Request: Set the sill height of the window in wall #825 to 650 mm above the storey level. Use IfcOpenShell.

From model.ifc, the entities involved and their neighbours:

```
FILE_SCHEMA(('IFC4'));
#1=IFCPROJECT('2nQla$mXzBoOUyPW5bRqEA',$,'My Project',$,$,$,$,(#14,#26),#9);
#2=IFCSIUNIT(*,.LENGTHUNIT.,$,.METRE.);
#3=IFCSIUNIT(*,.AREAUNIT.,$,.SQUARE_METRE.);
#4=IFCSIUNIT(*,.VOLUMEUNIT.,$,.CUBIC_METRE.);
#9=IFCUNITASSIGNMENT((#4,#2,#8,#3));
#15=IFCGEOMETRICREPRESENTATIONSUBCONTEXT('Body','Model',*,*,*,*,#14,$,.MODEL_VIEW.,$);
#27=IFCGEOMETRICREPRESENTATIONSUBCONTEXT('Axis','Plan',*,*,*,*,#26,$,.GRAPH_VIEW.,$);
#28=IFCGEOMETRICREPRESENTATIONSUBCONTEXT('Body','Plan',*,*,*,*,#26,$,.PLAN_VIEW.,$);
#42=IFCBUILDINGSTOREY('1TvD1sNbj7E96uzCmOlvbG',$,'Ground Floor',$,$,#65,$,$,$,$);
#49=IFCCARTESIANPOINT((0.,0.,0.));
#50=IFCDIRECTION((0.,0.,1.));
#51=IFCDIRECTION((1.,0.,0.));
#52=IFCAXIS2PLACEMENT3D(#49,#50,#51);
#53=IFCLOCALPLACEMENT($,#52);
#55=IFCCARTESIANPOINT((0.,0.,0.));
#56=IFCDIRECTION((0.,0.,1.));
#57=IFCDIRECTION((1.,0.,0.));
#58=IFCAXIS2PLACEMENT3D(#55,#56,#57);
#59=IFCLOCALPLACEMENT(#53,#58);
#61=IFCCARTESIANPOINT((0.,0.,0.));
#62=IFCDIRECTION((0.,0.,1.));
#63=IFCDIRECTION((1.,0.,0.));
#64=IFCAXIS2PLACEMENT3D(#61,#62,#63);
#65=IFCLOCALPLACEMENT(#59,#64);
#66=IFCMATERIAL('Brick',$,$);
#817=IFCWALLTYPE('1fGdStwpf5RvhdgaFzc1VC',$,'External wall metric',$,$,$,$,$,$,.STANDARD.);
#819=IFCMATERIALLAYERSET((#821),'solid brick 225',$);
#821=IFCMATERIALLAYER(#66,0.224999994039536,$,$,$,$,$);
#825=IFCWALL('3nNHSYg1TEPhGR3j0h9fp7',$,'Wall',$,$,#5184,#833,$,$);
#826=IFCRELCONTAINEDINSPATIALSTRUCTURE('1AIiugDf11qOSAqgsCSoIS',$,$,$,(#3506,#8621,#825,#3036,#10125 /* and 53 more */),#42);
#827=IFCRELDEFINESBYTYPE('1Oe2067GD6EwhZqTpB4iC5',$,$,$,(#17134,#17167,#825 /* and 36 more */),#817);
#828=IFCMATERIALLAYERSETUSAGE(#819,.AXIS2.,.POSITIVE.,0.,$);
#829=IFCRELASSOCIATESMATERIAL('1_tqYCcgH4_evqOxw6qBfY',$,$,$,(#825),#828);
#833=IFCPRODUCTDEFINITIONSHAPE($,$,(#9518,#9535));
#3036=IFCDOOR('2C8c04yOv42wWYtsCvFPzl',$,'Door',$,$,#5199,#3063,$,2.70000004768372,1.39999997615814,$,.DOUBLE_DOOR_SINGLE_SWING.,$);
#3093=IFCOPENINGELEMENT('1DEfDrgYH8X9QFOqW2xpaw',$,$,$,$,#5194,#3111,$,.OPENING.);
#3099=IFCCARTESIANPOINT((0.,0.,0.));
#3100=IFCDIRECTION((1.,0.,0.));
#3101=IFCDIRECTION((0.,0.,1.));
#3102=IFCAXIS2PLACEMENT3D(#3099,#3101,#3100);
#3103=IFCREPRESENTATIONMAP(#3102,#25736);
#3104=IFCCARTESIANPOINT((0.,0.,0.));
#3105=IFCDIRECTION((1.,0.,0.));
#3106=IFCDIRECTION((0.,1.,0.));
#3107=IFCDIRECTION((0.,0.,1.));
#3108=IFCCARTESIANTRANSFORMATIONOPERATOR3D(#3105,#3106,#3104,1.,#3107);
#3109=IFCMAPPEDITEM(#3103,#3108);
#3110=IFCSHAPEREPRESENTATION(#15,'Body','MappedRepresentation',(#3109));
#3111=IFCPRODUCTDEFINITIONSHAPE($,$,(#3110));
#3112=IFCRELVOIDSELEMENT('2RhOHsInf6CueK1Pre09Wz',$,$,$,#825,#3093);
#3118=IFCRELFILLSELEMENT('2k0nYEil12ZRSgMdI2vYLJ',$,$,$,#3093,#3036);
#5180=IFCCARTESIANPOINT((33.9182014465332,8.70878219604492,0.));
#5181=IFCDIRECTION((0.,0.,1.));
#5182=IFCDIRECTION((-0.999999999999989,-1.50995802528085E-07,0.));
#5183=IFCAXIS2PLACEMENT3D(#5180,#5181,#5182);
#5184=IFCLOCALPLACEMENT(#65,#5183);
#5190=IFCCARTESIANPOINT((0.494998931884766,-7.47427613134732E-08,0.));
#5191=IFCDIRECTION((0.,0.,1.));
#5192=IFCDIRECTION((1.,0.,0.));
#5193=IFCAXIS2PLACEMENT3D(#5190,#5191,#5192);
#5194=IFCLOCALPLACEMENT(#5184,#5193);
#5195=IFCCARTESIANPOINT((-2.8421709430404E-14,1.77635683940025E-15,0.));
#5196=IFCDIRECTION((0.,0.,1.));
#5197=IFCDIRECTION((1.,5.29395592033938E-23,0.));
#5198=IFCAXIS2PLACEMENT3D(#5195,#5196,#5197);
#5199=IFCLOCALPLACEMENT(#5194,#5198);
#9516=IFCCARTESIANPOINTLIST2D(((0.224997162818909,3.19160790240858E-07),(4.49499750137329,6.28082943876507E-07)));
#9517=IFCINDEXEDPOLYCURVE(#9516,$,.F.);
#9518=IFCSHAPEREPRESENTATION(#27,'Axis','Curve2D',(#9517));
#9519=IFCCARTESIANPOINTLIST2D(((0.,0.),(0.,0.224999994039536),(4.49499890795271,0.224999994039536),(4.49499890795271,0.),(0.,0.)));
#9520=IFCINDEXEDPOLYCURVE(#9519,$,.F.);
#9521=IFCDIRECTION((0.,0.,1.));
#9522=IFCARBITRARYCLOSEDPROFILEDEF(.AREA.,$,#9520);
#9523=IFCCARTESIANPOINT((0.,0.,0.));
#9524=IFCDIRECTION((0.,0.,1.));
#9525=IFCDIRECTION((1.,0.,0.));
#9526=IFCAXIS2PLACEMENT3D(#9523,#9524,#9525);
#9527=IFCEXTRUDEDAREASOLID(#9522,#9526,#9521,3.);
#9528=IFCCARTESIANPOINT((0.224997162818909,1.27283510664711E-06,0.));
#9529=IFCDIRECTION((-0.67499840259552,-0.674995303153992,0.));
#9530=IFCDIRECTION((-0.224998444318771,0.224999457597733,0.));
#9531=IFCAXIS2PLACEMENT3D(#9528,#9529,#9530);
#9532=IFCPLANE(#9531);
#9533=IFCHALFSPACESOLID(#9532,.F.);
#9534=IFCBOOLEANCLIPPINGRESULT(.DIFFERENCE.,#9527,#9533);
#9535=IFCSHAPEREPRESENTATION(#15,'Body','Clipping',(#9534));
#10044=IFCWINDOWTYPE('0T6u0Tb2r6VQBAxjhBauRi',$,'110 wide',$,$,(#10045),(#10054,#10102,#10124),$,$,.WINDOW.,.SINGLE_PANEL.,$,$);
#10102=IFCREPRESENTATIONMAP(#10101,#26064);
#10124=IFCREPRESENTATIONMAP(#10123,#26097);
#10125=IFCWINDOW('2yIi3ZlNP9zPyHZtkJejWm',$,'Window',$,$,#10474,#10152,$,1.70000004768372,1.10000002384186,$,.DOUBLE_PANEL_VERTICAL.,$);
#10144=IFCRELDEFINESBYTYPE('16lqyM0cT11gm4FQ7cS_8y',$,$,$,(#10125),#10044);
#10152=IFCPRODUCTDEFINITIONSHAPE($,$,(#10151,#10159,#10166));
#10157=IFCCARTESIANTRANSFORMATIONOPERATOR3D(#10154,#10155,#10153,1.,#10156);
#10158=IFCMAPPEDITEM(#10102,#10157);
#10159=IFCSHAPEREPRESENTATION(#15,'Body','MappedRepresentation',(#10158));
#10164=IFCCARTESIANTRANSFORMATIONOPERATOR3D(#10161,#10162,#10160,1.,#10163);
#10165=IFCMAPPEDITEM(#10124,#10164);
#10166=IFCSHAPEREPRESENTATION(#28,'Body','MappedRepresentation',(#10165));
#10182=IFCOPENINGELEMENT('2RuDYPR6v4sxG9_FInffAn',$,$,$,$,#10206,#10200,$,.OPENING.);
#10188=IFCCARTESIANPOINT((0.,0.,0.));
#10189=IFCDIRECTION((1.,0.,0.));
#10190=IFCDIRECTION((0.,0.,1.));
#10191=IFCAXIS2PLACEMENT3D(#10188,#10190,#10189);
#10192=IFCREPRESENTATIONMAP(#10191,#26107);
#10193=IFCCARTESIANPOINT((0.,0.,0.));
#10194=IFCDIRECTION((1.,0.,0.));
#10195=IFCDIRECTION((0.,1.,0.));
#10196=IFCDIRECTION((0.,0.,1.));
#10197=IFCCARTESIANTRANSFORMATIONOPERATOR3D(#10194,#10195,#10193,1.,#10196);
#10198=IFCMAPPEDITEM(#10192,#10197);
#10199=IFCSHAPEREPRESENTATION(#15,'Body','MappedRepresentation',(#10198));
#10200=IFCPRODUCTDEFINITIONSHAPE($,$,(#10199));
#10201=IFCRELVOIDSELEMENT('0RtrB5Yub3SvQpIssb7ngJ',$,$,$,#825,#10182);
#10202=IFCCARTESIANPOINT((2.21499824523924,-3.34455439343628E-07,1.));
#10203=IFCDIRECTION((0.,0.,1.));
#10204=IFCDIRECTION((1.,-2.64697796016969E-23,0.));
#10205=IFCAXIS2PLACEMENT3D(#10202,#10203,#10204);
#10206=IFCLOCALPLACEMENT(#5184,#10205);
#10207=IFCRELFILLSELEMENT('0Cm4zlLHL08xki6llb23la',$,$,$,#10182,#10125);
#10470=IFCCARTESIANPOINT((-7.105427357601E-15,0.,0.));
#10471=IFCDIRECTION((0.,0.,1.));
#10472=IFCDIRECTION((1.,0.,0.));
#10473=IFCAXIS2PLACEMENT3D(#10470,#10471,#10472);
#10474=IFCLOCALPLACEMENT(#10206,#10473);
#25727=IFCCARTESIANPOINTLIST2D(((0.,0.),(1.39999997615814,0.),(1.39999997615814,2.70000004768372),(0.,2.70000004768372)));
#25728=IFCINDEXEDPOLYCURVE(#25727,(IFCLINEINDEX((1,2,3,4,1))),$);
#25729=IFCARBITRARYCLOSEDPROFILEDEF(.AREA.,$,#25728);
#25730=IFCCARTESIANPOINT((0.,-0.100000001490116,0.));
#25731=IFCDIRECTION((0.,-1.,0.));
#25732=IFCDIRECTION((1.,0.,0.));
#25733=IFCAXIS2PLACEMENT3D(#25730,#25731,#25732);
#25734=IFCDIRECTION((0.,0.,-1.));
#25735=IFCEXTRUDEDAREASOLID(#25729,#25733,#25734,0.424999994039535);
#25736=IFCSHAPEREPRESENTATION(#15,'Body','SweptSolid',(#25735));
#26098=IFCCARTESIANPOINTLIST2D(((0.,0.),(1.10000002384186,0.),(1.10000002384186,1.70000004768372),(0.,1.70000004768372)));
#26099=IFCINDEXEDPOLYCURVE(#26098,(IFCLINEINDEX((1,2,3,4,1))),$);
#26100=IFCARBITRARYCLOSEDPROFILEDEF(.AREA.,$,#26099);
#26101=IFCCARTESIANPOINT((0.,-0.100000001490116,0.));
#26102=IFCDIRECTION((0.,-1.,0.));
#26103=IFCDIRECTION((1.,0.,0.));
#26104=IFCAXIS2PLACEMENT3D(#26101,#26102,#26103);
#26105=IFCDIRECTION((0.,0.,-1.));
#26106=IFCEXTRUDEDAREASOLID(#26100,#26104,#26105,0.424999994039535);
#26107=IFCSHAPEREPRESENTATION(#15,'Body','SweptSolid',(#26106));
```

```python
import numpy as np
import ifcopenshell
import ifcopenshell.api.geometry
import ifcopenshell.geom
import ifcopenshell.util.element
import ifcopenshell.util.placement
import ifcopenshell.util.shape
import ifcopenshell.util.unit

model = ifcopenshell.open("model.ifc")
unit_scale = ifcopenshell.util.unit.calculate_unit_scale(model)

window = model.by_guid("2yIi3ZlNP9zPyHZtkJejWm")
opening = window.FillsVoids[0].RelatingOpeningElement
storey = ifcopenshell.util.element.get_container(window, ifc_class="IfcBuildingStorey")
level = ifcopenshell.util.placement.get_local_placement(storey.ObjectPlacement)[2, 3]

# The opening's origin need not be at the sill, so measure its lowest point.
shape = ifcopenshell.geom.create_shape(ifcopenshell.geom.settings(), opening)
bottom = ifcopenshell.util.shape.get_shape_bottom_elevation(shape, shape.geometry) / unit_scale
dz = level + 0.65 / unit_scale - bottom

shift = np.array([0.0, 0.0, dz])
# The window is placed relative to its opening, so it follows when the opening moves.
matrix = ifcopenshell.util.placement.get_local_placement(opening.ObjectPlacement)
matrix[:3, 3] += shift
ifcopenshell.api.geometry.edit_object_placement(
    model, product=opening, matrix=matrix, is_si=False, should_transform_children=True
)

print(f"moved by {dz * unit_scale:+.3f} m")

model.write("model-out.ifc")
```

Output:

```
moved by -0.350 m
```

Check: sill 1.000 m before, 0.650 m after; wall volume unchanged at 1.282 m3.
